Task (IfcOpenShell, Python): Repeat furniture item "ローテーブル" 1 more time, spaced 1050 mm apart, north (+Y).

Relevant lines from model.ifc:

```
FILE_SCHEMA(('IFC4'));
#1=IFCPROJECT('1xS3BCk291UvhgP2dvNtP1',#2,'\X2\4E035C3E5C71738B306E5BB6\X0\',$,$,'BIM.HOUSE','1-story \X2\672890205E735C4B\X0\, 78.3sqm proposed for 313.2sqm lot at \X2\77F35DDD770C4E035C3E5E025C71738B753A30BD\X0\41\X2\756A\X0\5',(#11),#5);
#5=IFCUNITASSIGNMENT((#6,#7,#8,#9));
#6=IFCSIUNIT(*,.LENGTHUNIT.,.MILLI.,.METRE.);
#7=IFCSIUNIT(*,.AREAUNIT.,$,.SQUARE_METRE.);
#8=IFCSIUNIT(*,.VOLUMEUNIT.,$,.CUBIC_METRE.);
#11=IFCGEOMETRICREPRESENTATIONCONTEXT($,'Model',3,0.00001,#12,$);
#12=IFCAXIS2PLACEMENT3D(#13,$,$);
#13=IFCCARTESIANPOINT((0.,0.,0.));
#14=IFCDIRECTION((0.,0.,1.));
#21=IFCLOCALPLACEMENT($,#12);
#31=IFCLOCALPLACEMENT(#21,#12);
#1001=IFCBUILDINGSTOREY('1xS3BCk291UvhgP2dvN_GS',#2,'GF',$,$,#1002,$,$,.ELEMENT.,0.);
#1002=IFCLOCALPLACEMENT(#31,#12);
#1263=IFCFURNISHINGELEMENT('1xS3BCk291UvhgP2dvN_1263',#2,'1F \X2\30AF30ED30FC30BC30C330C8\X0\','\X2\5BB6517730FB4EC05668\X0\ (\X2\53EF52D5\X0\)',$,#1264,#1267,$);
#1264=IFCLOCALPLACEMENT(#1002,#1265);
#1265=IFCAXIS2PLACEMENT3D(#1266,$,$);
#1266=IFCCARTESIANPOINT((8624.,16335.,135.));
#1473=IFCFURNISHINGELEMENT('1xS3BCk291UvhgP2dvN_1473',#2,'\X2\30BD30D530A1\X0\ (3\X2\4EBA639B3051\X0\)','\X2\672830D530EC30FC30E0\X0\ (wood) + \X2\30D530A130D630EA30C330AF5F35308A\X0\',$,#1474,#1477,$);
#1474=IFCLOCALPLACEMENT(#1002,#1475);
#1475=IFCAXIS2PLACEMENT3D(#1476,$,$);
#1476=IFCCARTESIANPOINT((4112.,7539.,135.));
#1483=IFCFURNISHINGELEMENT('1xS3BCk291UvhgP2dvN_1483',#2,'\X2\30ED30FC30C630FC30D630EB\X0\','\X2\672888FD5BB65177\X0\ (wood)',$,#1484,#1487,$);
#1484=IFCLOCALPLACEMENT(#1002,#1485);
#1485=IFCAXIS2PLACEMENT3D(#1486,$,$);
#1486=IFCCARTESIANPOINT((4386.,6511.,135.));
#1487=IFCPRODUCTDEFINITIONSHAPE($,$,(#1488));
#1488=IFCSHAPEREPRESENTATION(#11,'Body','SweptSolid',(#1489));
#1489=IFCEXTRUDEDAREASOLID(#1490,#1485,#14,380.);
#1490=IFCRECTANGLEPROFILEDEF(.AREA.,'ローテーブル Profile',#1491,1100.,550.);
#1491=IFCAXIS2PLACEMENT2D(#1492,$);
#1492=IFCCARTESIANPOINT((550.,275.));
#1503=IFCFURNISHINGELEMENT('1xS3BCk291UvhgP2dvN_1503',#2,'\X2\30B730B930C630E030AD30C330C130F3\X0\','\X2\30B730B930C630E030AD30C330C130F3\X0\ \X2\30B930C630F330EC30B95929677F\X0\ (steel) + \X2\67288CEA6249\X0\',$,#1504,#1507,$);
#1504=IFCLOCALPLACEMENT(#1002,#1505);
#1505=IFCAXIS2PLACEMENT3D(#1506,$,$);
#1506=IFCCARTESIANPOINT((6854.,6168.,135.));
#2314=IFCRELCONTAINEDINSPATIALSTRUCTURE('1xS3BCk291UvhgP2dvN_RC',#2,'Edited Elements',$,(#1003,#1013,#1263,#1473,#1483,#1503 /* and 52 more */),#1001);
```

```python
import numpy as np
import ifcopenshell
import ifcopenshell.api.geometry
import ifcopenshell.api.root
import ifcopenshell.util.element
import ifcopenshell.util.placement

model = ifcopenshell.open("model.ifc")


def reuse_history(source, copy):
    """copy_class also copies each property set's owner history, people and application; keep the originals."""
    for rel in copy.IsDefinedBy:
        if rel.is_a("IfcRelDefinesByProperties") and (history := rel.RelatingPropertyDefinition.OwnerHistory):
            rel.RelatingPropertyDefinition.OwnerHistory = source.OwnerHistory
            ifcopenshell.util.element.remove_deep2(model, history)


source = model.by_guid("1xS3BCk291UvhgP2dvN_1483")
base = ifcopenshell.util.placement.get_local_placement(source.ObjectPlacement)
step = np.array([0.0, 1.0, 0.0]) * 1050.0

for i in range(1, 2):
    copy = ifcopenshell.api.root.copy_class(model, product=source)
    copy.Representation = ifcopenshell.util.element.copy_deep(
        model, source.Representation, exclude=["IfcGeometricRepresentationContext", "IfcRepresentationMap"]
    )
    reuse_history(source, copy)
    matrix = base.copy()
    matrix[:3, 3] += i * step
    print("added at", matrix[:3, 3].round(3) + 0.0)
    ifcopenshell.api.geometry.edit_object_placement(model, product=copy, matrix=matrix, is_si=False)

model.write("model-out.ifc")
```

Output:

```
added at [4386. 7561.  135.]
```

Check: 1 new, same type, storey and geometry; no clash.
